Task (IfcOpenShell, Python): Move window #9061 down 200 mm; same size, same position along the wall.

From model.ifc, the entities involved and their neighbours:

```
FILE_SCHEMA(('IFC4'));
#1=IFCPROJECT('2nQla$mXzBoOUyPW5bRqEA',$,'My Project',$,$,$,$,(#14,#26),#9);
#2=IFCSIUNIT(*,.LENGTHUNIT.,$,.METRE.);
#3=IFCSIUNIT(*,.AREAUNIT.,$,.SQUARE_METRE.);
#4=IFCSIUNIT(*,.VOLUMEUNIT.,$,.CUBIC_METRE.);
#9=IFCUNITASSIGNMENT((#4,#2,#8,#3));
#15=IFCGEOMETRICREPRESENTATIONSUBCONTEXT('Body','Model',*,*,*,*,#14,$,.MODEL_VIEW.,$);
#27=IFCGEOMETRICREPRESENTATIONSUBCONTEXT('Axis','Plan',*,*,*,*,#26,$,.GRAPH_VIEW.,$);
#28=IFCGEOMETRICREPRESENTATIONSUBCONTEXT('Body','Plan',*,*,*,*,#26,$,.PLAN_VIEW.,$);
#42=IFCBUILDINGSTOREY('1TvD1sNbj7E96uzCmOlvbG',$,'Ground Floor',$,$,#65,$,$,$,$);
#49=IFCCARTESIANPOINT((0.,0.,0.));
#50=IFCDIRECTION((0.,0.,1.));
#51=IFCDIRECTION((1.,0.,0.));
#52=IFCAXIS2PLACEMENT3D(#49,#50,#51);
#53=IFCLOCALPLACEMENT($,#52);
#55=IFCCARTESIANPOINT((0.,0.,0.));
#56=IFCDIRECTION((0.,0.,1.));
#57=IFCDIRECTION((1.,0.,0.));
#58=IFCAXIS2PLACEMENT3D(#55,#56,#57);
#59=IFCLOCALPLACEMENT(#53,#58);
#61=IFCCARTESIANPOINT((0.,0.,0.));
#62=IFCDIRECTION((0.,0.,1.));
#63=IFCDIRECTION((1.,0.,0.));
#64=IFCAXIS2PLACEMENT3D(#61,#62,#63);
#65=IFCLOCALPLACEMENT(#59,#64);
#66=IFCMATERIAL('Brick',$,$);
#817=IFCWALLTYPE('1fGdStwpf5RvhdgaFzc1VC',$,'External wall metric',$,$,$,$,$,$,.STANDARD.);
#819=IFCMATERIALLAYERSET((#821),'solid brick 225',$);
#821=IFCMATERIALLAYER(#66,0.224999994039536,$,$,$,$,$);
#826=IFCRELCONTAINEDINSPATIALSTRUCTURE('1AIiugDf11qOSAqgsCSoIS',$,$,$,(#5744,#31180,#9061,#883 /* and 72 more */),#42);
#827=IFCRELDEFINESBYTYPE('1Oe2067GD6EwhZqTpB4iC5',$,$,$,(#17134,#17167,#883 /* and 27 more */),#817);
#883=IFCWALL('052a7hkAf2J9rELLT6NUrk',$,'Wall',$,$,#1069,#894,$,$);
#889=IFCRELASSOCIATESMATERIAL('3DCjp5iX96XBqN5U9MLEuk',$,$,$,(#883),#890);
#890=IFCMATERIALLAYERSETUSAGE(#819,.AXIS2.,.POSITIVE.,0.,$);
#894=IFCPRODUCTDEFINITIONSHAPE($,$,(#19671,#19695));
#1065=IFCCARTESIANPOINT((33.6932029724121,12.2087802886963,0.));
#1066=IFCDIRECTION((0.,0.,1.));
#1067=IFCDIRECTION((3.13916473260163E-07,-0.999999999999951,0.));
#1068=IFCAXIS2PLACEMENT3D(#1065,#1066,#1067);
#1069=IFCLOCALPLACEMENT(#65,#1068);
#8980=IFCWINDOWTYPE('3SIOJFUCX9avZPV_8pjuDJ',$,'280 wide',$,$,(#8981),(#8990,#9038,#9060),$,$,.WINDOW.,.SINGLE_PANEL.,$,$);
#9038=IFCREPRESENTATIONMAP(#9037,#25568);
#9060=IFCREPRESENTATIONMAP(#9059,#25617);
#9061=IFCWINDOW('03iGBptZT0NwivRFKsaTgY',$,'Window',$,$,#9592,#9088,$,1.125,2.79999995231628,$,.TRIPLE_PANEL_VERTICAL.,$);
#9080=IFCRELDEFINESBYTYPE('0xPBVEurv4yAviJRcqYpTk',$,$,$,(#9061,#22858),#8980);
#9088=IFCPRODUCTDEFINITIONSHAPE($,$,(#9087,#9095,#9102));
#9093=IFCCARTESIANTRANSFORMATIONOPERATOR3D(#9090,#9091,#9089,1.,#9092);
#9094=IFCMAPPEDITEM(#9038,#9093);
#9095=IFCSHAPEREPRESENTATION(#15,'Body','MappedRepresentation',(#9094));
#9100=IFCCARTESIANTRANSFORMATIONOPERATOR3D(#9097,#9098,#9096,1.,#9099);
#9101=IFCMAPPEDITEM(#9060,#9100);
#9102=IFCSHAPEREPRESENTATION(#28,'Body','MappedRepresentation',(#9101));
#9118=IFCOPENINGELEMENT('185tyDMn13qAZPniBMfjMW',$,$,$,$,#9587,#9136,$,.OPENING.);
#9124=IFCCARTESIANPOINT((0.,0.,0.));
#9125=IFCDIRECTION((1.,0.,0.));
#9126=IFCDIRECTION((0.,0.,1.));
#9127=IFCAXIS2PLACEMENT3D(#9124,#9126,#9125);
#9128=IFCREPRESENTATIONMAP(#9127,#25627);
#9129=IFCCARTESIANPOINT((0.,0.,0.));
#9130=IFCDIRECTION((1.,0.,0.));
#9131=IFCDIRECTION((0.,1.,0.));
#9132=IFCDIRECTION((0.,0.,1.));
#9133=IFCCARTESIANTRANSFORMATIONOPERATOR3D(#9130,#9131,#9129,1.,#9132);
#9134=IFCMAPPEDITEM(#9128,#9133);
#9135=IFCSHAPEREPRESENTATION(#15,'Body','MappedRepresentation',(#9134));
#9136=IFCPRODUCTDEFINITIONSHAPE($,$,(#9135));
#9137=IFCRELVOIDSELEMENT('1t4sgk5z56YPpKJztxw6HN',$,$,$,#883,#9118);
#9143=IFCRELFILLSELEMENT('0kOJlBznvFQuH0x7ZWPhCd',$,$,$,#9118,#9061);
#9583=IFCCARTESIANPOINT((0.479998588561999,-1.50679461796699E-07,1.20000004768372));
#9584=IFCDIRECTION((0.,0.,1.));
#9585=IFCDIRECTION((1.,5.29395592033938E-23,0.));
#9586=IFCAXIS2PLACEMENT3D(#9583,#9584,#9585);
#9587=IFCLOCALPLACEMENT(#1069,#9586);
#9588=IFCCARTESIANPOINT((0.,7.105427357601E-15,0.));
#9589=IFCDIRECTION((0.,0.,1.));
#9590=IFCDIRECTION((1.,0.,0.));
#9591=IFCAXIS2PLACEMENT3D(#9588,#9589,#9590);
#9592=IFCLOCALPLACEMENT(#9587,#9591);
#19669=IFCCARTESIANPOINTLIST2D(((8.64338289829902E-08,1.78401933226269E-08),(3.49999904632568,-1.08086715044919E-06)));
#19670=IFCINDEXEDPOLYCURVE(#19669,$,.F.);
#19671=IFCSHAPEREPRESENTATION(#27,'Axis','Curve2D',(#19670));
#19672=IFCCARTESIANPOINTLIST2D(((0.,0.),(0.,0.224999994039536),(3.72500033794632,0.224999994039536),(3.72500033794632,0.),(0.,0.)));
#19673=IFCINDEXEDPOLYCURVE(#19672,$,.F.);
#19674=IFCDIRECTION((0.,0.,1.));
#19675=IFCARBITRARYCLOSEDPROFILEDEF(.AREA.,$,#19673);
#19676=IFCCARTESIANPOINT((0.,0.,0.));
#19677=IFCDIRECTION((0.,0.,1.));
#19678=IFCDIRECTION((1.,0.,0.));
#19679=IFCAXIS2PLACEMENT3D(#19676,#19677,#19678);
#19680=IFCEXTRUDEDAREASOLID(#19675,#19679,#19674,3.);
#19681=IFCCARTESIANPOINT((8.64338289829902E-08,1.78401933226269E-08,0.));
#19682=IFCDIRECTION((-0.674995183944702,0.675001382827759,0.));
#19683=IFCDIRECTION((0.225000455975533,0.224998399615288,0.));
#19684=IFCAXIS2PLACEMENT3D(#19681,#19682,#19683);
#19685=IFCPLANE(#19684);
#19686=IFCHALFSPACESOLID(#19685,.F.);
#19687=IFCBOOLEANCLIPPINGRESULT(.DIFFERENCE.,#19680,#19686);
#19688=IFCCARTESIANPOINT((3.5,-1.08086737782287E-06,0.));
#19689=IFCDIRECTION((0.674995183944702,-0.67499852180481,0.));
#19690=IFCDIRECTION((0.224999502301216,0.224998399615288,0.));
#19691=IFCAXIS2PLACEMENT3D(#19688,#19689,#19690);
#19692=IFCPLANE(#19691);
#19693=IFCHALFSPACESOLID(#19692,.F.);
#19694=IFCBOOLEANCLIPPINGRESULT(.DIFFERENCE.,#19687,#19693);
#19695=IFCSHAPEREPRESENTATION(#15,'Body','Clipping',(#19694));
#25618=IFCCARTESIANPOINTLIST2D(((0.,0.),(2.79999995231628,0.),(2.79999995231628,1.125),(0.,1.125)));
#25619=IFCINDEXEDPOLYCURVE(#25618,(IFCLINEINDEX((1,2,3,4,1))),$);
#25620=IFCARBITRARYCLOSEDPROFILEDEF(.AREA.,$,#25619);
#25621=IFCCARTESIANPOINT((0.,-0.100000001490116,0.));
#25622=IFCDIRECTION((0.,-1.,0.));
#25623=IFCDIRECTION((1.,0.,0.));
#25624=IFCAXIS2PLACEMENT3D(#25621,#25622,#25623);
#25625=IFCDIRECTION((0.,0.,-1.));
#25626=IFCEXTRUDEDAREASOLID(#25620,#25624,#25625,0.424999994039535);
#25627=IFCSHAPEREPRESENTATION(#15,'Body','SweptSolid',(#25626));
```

```python
import numpy as np
import ifcopenshell
import ifcopenshell.api.geometry
import ifcopenshell.util.placement
import ifcopenshell.util.unit

model = ifcopenshell.open("model.ifc")
unit_scale = ifcopenshell.util.unit.calculate_unit_scale(model)

window = model.by_guid("03iGBptZT0NwivRFKsaTgY")
opening = window.FillsVoids[0].RelatingOpeningElement
dz = -0.2 / unit_scale

shift = np.array([0.0, 0.0, dz])
# The window is placed relative to its opening, so it follows when the opening moves.
matrix = ifcopenshell.util.placement.get_local_placement(opening.ObjectPlacement)
matrix[:3, 3] += shift
ifcopenshell.api.geometry.edit_object_placement(
    model, product=opening, matrix=matrix, is_si=False, should_transform_children=True
)

print(f"moved by {dz * unit_scale:+.3f} m")

model.write("model_rev.ifc")
```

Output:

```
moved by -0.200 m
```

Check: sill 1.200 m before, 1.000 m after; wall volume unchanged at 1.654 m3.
